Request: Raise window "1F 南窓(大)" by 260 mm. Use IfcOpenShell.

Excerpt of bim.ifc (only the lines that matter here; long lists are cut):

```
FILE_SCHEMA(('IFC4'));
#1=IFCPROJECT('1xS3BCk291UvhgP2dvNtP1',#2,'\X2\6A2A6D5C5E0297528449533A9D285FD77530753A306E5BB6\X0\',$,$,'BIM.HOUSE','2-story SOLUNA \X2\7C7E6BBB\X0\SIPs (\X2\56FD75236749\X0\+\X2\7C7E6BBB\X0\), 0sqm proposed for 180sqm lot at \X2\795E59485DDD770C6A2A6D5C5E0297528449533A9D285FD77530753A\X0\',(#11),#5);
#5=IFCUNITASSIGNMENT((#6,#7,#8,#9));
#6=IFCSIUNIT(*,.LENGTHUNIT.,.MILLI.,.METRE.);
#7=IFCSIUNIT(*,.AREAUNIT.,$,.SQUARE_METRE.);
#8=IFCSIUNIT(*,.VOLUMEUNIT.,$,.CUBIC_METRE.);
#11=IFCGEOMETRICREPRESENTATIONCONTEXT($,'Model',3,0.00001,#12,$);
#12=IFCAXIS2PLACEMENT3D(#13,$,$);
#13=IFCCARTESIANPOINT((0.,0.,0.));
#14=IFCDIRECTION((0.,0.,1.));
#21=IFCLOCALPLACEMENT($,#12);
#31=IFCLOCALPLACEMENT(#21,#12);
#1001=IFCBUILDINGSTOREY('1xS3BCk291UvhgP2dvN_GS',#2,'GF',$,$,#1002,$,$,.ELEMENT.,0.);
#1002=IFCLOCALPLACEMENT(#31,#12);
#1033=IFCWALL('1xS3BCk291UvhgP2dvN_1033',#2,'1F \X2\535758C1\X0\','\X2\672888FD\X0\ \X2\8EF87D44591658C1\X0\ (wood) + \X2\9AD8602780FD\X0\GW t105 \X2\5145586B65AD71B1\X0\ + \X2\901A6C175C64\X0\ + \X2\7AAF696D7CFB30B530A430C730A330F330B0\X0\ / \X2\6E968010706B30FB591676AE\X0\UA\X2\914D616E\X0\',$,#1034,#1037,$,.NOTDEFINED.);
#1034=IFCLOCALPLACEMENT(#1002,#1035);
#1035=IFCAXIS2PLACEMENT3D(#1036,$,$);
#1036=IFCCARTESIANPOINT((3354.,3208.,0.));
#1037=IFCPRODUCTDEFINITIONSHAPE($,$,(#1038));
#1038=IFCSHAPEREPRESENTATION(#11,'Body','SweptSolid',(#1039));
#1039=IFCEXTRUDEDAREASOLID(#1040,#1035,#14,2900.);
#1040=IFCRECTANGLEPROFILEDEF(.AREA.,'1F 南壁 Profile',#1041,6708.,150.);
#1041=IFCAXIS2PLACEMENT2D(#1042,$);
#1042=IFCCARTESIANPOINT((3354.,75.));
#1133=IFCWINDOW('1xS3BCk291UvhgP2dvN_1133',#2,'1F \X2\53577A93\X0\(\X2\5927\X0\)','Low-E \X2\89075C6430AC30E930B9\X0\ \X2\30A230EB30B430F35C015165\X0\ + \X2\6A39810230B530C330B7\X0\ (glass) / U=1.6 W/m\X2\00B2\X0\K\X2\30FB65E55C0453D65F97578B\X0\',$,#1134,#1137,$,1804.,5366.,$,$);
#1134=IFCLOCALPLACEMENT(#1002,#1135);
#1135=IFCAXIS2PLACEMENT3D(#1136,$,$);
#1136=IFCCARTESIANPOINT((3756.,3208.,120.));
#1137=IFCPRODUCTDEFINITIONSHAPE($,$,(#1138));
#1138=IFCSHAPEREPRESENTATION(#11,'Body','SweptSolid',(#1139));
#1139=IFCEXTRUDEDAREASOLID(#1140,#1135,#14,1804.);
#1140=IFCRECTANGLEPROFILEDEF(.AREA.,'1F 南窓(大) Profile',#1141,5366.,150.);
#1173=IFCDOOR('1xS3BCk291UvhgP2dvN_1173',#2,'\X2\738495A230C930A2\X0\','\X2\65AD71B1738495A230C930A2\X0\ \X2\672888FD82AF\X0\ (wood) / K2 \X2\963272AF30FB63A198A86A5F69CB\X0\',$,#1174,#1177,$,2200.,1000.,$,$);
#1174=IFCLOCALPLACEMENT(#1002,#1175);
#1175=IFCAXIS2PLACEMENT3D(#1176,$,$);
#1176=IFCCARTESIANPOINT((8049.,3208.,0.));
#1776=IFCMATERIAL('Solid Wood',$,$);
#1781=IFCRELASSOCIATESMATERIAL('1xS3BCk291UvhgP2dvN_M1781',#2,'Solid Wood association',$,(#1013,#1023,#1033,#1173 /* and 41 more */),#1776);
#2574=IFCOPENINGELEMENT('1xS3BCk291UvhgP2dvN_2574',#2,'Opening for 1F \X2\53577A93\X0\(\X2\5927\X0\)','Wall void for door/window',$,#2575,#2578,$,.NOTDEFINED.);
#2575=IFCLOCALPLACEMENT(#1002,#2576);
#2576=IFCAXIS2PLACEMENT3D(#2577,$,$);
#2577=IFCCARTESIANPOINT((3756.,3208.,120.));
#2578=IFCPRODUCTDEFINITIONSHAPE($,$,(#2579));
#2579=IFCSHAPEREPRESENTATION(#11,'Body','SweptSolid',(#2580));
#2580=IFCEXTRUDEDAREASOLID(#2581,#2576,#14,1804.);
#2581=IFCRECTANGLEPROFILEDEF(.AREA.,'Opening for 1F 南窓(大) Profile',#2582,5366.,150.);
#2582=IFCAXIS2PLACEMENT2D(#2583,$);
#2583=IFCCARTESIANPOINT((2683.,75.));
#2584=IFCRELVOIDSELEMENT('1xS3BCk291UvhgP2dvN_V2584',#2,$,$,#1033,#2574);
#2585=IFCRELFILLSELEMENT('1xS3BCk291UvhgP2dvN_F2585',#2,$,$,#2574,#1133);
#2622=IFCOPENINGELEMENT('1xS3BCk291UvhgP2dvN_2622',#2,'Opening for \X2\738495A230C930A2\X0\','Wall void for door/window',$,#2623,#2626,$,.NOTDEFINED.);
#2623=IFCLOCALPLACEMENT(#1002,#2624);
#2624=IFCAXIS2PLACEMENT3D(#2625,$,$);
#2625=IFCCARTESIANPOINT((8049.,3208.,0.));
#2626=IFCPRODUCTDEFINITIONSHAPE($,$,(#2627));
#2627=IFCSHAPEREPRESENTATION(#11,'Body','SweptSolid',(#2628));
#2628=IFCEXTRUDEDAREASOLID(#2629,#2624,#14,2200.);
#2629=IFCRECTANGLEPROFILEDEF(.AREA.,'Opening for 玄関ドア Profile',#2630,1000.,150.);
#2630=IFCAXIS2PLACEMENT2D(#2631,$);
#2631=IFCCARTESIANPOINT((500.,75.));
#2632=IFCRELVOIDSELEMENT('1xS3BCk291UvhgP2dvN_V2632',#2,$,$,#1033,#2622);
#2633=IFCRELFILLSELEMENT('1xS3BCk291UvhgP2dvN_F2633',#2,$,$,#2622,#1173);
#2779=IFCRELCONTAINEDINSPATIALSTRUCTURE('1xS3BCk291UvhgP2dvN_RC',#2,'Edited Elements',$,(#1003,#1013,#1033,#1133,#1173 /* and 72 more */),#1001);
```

```python
import numpy as np
import ifcopenshell
import ifcopenshell.api.geometry
import ifcopenshell.util.placement
import ifcopenshell.util.unit

model = ifcopenshell.open("bim.ifc")
unit_scale = ifcopenshell.util.unit.calculate_unit_scale(model)

window = model.by_id(1133)
opening = window.FillsVoids[0].RelatingOpeningElement
dz = 260.0

shift = np.array([0.0, 0.0, dz])
# The window is not placed relative to its opening, so move both.
for product in (opening, window):
    matrix = ifcopenshell.util.placement.get_local_placement(product.ObjectPlacement)
    matrix[:3, 3] += shift
    ifcopenshell.api.geometry.edit_object_placement(model, product=product, matrix=matrix, is_si=False)

print(f"moved by {dz * unit_scale:+.3f} m")

model.write("bim_edited.ifc")
```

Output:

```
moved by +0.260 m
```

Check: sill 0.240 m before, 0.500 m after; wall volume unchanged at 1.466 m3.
